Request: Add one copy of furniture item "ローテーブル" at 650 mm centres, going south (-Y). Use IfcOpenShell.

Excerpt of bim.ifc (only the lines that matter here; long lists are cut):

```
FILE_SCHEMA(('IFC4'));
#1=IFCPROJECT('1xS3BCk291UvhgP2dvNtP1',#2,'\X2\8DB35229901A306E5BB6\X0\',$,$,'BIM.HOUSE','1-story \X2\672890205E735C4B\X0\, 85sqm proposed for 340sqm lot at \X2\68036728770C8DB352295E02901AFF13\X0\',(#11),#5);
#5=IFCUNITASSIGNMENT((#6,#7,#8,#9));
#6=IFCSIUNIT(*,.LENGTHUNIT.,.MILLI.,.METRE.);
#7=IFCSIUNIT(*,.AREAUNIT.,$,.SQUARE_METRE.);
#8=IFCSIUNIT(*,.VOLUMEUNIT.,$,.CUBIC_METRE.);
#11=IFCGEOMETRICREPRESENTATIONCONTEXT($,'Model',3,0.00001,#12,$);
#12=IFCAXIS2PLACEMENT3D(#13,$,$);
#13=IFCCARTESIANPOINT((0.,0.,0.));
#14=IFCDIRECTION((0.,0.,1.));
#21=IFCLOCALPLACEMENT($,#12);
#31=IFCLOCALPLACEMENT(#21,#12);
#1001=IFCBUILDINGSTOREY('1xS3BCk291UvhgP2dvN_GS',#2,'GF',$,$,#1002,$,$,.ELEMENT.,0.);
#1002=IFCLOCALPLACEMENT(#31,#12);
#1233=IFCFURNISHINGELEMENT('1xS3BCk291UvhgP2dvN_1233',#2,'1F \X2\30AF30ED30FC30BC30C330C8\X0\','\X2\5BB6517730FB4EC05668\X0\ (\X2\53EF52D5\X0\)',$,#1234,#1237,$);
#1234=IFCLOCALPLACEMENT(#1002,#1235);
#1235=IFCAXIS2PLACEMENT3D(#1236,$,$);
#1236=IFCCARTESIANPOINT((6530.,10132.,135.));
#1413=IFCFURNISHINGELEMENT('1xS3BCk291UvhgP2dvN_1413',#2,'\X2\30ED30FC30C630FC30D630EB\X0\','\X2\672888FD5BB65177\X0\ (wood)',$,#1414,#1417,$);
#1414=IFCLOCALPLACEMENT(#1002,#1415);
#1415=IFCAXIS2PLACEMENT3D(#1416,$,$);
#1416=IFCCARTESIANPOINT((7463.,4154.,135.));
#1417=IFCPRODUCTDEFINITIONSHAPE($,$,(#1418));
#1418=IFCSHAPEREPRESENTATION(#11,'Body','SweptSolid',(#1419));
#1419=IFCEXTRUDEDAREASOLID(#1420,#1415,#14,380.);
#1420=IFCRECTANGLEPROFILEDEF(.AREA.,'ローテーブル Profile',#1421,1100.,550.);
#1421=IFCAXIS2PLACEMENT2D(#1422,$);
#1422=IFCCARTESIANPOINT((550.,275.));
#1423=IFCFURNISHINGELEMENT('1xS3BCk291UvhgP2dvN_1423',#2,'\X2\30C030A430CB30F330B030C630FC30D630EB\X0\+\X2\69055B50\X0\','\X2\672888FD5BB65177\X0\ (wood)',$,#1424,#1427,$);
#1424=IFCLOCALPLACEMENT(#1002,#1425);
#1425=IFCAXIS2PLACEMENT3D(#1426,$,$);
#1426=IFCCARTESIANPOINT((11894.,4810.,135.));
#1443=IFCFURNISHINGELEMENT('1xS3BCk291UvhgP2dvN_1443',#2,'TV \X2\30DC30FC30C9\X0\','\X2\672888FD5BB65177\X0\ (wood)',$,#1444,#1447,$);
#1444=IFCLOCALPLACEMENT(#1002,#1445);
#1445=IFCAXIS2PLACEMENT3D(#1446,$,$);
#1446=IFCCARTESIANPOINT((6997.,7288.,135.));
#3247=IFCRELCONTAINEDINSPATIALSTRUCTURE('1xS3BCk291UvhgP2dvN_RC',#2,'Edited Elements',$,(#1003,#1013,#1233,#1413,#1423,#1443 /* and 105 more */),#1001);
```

```python
import numpy as np
import ifcopenshell
import ifcopenshell.api.geometry
import ifcopenshell.api.root
import ifcopenshell.util.element
import ifcopenshell.util.placement

model = ifcopenshell.open("bim.ifc")


def reuse_history(source, copy):
    """copy_class also copies each property set's owner history, people and application; keep the originals."""
    for rel in copy.IsDefinedBy:
        if rel.is_a("IfcRelDefinesByProperties") and (history := rel.RelatingPropertyDefinition.OwnerHistory):
            rel.RelatingPropertyDefinition.OwnerHistory = source.OwnerHistory
            ifcopenshell.util.element.remove_deep2(model, history)


source = model.by_guid("1xS3BCk291UvhgP2dvN_1413")
base = ifcopenshell.util.placement.get_local_placement(source.ObjectPlacement)
step = np.array([0.0, -1.0, 0.0]) * 650.0

for i in range(1, 2):
    copy = ifcopenshell.api.root.copy_class(model, product=source)
    copy.Representation = ifcopenshell.util.element.copy_deep(
        model, source.Representation, exclude=["IfcGeometricRepresentationContext", "IfcRepresentationMap"]
    )
    reuse_history(source, copy)
    matrix = base.copy()
    matrix[:3, 3] += i * step
    print("added at", matrix[:3, 3].round(3) + 0.0)
    ifcopenshell.api.geometry.edit_object_placement(model, product=copy, matrix=matrix, is_si=False)

model.write("bim-out.ifc")
```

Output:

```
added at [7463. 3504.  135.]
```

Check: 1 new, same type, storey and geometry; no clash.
